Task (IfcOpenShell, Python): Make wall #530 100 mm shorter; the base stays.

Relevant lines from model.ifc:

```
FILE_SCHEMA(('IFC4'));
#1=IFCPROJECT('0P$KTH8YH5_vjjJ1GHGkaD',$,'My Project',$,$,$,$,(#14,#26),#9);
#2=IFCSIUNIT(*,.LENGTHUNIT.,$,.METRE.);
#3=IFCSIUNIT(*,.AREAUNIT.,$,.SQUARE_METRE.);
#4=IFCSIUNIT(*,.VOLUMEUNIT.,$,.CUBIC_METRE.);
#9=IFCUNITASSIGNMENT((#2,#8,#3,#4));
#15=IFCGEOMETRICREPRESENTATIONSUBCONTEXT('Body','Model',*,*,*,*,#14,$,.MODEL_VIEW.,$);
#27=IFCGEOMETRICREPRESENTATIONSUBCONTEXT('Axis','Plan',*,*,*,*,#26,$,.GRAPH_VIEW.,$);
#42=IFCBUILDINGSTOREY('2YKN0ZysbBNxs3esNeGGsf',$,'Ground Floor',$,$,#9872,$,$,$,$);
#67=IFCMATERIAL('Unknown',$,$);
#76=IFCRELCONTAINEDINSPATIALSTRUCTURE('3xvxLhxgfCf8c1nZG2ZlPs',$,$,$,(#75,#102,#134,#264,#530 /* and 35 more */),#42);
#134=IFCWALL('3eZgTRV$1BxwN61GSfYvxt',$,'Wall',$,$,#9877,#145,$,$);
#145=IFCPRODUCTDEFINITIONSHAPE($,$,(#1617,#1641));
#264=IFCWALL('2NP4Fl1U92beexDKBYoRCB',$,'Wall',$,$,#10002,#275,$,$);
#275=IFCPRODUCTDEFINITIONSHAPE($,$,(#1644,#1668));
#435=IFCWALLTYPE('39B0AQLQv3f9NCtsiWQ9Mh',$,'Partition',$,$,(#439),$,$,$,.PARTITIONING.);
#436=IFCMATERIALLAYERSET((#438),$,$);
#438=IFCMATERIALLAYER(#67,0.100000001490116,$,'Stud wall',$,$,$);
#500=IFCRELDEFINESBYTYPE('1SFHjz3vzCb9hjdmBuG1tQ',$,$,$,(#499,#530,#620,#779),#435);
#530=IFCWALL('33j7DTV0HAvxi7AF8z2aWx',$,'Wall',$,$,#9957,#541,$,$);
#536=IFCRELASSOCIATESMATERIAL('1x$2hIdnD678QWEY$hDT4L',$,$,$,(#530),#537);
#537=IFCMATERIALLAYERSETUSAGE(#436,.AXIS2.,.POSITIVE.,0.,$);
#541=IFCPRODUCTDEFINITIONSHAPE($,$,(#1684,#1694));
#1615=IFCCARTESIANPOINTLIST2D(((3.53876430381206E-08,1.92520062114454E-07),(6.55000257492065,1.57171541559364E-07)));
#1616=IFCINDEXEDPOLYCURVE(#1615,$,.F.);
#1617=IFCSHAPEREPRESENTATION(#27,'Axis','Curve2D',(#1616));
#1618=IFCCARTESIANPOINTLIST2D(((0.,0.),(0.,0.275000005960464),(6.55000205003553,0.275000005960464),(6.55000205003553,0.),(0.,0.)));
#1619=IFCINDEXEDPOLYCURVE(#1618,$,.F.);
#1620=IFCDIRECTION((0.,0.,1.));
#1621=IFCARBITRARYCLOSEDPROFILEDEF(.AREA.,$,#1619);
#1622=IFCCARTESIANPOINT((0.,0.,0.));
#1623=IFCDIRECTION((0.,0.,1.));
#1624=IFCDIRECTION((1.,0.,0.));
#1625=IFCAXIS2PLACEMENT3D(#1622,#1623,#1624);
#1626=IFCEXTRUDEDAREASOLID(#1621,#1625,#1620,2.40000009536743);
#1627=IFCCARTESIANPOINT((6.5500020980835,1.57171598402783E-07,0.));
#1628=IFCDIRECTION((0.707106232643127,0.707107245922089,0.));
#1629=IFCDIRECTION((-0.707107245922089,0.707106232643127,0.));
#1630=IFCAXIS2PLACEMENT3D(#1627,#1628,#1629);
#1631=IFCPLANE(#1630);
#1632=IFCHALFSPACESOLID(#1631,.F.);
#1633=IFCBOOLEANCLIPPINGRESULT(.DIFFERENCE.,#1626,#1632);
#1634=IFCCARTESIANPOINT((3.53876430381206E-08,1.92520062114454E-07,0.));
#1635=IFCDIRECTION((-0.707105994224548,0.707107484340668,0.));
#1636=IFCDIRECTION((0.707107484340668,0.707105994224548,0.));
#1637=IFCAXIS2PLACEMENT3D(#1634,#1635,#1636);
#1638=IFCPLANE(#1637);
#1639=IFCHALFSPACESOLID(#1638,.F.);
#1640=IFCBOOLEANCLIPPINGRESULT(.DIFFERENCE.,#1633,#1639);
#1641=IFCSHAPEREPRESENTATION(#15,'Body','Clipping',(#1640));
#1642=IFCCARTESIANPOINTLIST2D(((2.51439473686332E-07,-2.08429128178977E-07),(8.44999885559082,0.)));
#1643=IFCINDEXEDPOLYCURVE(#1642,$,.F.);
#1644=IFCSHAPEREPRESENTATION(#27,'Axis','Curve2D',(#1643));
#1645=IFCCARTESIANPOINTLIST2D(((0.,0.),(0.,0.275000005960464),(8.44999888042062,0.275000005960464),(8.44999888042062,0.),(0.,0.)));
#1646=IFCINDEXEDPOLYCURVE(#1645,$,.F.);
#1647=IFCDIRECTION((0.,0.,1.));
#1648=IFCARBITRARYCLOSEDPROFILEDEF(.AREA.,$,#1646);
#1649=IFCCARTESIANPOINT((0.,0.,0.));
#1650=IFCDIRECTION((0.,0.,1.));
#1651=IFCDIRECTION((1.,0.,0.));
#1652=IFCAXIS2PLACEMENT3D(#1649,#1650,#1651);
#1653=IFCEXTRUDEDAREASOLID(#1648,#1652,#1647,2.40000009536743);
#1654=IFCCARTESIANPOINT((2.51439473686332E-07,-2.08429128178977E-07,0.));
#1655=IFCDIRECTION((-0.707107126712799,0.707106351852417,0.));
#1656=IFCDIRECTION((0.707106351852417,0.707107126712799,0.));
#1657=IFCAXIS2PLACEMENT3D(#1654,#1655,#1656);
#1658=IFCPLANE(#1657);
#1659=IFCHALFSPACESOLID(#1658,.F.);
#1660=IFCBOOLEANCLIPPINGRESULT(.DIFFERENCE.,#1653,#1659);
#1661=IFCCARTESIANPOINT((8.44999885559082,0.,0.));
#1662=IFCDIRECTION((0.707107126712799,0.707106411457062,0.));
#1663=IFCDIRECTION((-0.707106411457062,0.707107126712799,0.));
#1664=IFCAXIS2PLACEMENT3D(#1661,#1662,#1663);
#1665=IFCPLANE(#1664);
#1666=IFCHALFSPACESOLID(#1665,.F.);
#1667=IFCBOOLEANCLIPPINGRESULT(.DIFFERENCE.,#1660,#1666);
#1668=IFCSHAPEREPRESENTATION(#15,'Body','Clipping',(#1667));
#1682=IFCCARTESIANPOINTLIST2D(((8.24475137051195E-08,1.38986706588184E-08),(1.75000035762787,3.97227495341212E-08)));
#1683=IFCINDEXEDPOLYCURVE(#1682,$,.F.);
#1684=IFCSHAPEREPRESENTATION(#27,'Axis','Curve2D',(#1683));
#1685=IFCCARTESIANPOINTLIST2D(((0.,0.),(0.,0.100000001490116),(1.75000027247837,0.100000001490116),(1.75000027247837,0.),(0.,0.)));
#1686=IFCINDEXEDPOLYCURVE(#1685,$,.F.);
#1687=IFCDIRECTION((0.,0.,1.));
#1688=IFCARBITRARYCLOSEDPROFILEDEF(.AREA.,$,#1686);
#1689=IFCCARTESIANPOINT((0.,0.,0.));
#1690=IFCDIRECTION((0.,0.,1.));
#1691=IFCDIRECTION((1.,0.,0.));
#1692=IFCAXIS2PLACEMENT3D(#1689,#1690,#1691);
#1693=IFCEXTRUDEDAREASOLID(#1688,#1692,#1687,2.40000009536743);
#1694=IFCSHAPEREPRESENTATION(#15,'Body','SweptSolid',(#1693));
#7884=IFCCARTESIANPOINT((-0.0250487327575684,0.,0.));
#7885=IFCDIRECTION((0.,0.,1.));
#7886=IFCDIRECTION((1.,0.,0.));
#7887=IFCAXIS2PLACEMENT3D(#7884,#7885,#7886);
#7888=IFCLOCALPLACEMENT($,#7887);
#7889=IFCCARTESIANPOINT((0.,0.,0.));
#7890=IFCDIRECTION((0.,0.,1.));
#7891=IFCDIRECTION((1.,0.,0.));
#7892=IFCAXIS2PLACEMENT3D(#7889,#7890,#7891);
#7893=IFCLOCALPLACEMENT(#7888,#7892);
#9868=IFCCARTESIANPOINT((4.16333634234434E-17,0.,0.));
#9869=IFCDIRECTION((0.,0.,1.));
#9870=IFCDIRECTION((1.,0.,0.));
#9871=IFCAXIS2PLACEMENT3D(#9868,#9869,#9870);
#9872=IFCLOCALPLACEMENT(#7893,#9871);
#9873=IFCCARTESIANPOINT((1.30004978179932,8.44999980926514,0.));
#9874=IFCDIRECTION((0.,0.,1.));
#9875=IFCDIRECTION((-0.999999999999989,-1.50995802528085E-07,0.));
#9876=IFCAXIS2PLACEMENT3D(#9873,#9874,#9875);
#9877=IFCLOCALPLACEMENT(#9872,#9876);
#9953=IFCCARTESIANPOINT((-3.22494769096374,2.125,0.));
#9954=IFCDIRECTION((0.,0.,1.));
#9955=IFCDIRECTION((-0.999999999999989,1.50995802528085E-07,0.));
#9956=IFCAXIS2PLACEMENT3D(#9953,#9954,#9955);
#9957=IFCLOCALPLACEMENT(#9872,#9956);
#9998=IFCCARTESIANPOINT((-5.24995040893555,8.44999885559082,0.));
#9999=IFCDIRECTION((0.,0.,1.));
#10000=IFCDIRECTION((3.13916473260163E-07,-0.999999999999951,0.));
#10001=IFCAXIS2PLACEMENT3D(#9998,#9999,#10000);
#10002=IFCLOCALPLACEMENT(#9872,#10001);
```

```python
import ifcopenshell
import ifcopenshell.geom
import ifcopenshell.util.representation
import ifcopenshell.util.shape

model = ifcopenshell.open("model.ifc")
settings = ifcopenshell.geom.settings()


def volume(element):
    """Net volume in cubic metres, openings subtracted."""
    shape = ifcopenshell.geom.create_shape(settings, element)
    return ifcopenshell.util.shape.get_volume(shape.geometry)


wall = model.by_id(530)
before = volume(wall)

body = ifcopenshell.util.representation.get_representation(wall, "Model", "Body")
solid = body.Items[0]
old_height = solid.Depth
solid.Depth -= 0.1
after = volume(wall)

print(f"height {old_height:g} -> {solid.Depth:g}, volume {before:.3f} -> {after:.3f} m3")

model.write("model_rev.ifc")
```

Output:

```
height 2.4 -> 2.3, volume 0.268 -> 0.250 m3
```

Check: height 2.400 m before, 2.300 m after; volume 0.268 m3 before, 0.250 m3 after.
